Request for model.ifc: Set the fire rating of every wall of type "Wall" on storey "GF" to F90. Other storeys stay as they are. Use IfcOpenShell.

First a look at what the model holds.

```python
import ifcopenshell
import ifcopenshell.util.element

model = ifcopenshell.open("model.ifc")
print(model.schema)
storey = next(s for s in model.by_type("IfcBuildingStorey") if s.Name == "GF")
walls = [e for e in ifcopenshell.util.element.get_decomposition(storey) if e.is_a("IfcWall")]
seen = {}
for e in walls:
    element_type = ifcopenshell.util.element.get_type(e)
    key = (element_type.Name if element_type != e and element_type else None, ifcopenshell.util.element.get_pset(e, "Pset_WallCommon", "FireRating"))
    seen[key] = seen.get(key, 0) + 1
for (name, value), count in sorted(seen.items(), key=str):
    print(count, "x", name, "|", value)
```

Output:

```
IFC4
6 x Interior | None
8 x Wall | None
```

```python
import ifcopenshell
import ifcopenshell.api.pset
import ifcopenshell.util.element

model = ifcopenshell.open("model.ifc")

storey = next(s for s in model.by_type("IfcBuildingStorey") if s.Name == "GF")
walls = [e for e in ifcopenshell.util.element.get_decomposition(storey) if e.is_a("IfcWall")]

count = 0
for e in walls:
    element_type = ifcopenshell.util.element.get_type(e)
    if element_type in (None, e) or element_type.Name != "Wall":
        continue
    # add_pset returns the element's existing set when there is one.
    pset = ifcopenshell.api.pset.add_pset(model, product=e, name="Pset_WallCommon")
    ifcopenshell.api.pset.edit_pset(model, pset=pset, properties={"FireRating": "F90"})
    count += 1

print(count, "walls updated")

model.write("model-out.ifc")
```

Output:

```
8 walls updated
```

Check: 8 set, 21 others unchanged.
